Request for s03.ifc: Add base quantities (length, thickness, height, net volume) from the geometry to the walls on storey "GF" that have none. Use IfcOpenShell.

First a look at what the model holds.

```python
import ifcopenshell
import ifcopenshell.util.element
import ifcopenshell.util.unit

model = ifcopenshell.open("s03.ifc")
print(model.schema)
for unit_type in ("LENGTHUNIT", "AREAUNIT", "VOLUMEUNIT"):
    print(unit_type, ifcopenshell.util.unit.calculate_unit_scale(model, unit_type))
storey = next(s for s in model.by_type("IfcBuildingStorey") if s.Name == "GF")
walls = [e for e in ifcopenshell.util.element.get_decomposition(storey) if e.is_a("IfcWall")]
for e in sorted(walls, key=lambda e: e.id()):
    print(e.id(), e.is_a(), e.Name, list(ifcopenshell.util.element.get_psets(e, qtos_only=True)), sep=" | ")
```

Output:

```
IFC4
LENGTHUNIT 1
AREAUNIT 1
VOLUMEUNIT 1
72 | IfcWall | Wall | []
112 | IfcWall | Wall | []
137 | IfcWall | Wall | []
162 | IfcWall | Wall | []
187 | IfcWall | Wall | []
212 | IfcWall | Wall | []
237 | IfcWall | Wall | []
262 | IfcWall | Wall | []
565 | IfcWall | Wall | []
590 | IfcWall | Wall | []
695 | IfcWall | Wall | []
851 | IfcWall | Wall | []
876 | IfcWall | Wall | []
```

```python
import ifcopenshell
import ifcopenshell.api.pset
import ifcopenshell.geom
import ifcopenshell.util.element
import ifcopenshell.util.shape
import ifcopenshell.util.unit

model = ifcopenshell.open("s03.ifc")
unit_scale = ifcopenshell.util.unit.calculate_unit_scale(model)
volume_scale = ifcopenshell.util.unit.calculate_unit_scale(model, "VOLUMEUNIT")
settings = ifcopenshell.geom.settings()

storey = next(s for s in model.by_type("IfcBuildingStorey") if s.Name == "GF")
walls = [e for e in ifcopenshell.util.element.get_decomposition(storey) if e.is_a("IfcWall")]

for e in sorted(walls, key=lambda e: e.id()):
    if ifcopenshell.util.element.get_psets(e, qtos_only=True, should_inherit=False):
        continue
    # Geometry comes back in metres, in the element's own axes.
    shape = ifcopenshell.geom.create_shape(settings, e)
    values = {
        "Length": ifcopenshell.util.shape.get_x(shape.geometry) / unit_scale,
        "Width": ifcopenshell.util.shape.get_y(shape.geometry) / unit_scale,
        "Height": ifcopenshell.util.shape.get_z(shape.geometry) / unit_scale,
        "NetVolume": ifcopenshell.util.shape.get_volume(shape.geometry) / volume_scale,
    }
    qto = ifcopenshell.api.pset.add_qto(model, product=e, name="Qto_WallBaseQuantities")
    ifcopenshell.api.pset.edit_qto(model, qto=qto, properties=values)
    print(e.id(), {k: round(v, 3) for k, v in values.items()})

model.write("s03_updated.ifc")
```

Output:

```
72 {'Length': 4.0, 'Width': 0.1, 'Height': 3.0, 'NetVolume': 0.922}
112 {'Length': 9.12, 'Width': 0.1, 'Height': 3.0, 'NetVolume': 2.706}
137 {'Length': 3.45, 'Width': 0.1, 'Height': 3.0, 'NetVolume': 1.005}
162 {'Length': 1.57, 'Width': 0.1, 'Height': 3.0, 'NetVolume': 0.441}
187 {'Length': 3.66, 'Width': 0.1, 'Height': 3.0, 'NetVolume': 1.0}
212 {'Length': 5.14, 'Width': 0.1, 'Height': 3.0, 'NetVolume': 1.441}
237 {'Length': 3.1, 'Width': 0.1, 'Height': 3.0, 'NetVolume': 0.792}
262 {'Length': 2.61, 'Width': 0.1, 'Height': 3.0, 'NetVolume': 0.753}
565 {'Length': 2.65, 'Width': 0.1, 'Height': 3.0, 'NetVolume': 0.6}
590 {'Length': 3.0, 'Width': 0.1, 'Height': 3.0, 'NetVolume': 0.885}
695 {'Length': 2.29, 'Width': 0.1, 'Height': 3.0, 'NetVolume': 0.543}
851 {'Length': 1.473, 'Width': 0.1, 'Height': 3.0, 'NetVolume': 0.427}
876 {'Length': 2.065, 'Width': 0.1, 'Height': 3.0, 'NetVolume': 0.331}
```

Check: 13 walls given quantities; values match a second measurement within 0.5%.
